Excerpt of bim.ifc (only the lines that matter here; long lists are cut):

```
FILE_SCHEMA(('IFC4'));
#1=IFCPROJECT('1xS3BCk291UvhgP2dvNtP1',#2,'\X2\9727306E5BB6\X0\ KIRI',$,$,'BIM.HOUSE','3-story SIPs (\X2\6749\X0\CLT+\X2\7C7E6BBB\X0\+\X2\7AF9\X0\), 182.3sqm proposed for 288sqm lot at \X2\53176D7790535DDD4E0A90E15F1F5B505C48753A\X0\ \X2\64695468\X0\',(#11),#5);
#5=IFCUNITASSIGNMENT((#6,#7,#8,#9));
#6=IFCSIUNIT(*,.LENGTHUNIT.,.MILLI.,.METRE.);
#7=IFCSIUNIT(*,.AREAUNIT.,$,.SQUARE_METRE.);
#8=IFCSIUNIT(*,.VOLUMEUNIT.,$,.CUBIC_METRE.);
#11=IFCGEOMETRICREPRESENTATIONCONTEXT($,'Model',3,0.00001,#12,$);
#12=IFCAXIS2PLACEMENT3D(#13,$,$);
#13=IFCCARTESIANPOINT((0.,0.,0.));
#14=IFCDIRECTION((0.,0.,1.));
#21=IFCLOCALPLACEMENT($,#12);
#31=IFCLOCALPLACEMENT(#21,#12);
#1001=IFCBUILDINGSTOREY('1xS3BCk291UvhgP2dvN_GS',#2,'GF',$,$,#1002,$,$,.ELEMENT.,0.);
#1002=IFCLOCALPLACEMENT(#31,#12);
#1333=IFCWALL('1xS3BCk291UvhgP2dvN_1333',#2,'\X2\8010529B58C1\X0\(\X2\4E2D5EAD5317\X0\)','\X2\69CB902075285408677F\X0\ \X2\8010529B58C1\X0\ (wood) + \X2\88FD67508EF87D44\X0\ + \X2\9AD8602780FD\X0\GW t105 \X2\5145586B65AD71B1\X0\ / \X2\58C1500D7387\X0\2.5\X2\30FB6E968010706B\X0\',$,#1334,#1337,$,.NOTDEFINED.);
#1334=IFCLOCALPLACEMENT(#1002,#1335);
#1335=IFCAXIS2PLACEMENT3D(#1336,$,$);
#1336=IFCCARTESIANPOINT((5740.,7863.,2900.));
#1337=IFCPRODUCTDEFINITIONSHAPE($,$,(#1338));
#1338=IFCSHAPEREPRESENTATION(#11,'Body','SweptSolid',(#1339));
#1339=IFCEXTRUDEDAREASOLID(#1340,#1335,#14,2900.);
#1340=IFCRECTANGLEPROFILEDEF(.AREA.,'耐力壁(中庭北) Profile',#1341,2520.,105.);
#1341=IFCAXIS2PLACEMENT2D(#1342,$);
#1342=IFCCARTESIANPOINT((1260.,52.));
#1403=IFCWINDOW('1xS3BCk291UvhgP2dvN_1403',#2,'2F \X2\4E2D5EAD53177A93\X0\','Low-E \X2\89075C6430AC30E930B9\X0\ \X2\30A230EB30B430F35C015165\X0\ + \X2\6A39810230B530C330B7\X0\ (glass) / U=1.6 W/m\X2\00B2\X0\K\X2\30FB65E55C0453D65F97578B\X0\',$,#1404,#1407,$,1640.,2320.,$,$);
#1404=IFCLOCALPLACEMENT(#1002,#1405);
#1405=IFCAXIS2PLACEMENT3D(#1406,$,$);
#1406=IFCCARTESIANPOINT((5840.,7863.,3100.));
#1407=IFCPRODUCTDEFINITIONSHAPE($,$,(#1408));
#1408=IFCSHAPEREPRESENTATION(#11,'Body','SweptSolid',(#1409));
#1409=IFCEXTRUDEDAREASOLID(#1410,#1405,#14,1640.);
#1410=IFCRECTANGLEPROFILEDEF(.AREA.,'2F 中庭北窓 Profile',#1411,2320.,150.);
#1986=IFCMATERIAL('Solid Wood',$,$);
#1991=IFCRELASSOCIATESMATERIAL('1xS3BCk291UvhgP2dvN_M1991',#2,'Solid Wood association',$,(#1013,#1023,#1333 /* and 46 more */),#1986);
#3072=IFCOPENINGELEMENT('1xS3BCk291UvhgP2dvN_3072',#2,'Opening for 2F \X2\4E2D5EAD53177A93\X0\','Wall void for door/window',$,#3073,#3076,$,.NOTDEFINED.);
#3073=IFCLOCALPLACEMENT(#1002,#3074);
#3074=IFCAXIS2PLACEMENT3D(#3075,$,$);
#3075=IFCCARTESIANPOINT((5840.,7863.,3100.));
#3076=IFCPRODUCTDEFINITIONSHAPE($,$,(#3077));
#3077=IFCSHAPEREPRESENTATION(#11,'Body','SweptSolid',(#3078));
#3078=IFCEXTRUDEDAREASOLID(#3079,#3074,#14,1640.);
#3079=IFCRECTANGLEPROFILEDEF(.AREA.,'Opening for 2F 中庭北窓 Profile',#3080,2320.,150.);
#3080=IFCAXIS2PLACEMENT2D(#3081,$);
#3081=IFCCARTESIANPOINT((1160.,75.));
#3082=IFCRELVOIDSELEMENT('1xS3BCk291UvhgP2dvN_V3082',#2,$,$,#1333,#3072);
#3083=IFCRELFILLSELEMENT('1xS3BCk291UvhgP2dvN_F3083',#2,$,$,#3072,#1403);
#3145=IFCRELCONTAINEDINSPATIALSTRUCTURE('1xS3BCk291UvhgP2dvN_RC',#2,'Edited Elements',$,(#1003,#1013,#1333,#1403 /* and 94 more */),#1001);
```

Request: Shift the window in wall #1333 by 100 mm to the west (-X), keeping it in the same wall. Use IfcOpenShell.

```python
import ifcopenshell
import ifcopenshell.api.geometry
import ifcopenshell.util.placement
import ifcopenshell.util.unit

model = ifcopenshell.open("bim.ifc")
unit_scale = ifcopenshell.util.unit.calculate_unit_scale(model)

window = model.by_guid("1xS3BCk291UvhgP2dvN_1403")
opening = window.FillsVoids[0].RelatingOpeningElement
wall = opening.VoidsElements[0].RelatingBuildingElement

wall_matrix = ifcopenshell.util.placement.get_local_placement(wall.ObjectPlacement)
shift = wall_matrix[:3, 0] * -0.1 / unit_scale
before = ifcopenshell.util.placement.get_local_placement(window.ObjectPlacement)[:3, 3].copy()

# The window is not placed relative to its opening, so move both.
for product in (opening, window):
    matrix = ifcopenshell.util.placement.get_local_placement(product.ObjectPlacement)
    matrix[:3, 3] += shift
    ifcopenshell.api.geometry.edit_object_placement(model, product=product, matrix=matrix, is_si=False)

after = ifcopenshell.util.placement.get_local_placement(window.ObjectPlacement)[:3, 3]
print("window moved by", (after - before).round(3) + 0.0)

model.write("bim-out.ifc")
```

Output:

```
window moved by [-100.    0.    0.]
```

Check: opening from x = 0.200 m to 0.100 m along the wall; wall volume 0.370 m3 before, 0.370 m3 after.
